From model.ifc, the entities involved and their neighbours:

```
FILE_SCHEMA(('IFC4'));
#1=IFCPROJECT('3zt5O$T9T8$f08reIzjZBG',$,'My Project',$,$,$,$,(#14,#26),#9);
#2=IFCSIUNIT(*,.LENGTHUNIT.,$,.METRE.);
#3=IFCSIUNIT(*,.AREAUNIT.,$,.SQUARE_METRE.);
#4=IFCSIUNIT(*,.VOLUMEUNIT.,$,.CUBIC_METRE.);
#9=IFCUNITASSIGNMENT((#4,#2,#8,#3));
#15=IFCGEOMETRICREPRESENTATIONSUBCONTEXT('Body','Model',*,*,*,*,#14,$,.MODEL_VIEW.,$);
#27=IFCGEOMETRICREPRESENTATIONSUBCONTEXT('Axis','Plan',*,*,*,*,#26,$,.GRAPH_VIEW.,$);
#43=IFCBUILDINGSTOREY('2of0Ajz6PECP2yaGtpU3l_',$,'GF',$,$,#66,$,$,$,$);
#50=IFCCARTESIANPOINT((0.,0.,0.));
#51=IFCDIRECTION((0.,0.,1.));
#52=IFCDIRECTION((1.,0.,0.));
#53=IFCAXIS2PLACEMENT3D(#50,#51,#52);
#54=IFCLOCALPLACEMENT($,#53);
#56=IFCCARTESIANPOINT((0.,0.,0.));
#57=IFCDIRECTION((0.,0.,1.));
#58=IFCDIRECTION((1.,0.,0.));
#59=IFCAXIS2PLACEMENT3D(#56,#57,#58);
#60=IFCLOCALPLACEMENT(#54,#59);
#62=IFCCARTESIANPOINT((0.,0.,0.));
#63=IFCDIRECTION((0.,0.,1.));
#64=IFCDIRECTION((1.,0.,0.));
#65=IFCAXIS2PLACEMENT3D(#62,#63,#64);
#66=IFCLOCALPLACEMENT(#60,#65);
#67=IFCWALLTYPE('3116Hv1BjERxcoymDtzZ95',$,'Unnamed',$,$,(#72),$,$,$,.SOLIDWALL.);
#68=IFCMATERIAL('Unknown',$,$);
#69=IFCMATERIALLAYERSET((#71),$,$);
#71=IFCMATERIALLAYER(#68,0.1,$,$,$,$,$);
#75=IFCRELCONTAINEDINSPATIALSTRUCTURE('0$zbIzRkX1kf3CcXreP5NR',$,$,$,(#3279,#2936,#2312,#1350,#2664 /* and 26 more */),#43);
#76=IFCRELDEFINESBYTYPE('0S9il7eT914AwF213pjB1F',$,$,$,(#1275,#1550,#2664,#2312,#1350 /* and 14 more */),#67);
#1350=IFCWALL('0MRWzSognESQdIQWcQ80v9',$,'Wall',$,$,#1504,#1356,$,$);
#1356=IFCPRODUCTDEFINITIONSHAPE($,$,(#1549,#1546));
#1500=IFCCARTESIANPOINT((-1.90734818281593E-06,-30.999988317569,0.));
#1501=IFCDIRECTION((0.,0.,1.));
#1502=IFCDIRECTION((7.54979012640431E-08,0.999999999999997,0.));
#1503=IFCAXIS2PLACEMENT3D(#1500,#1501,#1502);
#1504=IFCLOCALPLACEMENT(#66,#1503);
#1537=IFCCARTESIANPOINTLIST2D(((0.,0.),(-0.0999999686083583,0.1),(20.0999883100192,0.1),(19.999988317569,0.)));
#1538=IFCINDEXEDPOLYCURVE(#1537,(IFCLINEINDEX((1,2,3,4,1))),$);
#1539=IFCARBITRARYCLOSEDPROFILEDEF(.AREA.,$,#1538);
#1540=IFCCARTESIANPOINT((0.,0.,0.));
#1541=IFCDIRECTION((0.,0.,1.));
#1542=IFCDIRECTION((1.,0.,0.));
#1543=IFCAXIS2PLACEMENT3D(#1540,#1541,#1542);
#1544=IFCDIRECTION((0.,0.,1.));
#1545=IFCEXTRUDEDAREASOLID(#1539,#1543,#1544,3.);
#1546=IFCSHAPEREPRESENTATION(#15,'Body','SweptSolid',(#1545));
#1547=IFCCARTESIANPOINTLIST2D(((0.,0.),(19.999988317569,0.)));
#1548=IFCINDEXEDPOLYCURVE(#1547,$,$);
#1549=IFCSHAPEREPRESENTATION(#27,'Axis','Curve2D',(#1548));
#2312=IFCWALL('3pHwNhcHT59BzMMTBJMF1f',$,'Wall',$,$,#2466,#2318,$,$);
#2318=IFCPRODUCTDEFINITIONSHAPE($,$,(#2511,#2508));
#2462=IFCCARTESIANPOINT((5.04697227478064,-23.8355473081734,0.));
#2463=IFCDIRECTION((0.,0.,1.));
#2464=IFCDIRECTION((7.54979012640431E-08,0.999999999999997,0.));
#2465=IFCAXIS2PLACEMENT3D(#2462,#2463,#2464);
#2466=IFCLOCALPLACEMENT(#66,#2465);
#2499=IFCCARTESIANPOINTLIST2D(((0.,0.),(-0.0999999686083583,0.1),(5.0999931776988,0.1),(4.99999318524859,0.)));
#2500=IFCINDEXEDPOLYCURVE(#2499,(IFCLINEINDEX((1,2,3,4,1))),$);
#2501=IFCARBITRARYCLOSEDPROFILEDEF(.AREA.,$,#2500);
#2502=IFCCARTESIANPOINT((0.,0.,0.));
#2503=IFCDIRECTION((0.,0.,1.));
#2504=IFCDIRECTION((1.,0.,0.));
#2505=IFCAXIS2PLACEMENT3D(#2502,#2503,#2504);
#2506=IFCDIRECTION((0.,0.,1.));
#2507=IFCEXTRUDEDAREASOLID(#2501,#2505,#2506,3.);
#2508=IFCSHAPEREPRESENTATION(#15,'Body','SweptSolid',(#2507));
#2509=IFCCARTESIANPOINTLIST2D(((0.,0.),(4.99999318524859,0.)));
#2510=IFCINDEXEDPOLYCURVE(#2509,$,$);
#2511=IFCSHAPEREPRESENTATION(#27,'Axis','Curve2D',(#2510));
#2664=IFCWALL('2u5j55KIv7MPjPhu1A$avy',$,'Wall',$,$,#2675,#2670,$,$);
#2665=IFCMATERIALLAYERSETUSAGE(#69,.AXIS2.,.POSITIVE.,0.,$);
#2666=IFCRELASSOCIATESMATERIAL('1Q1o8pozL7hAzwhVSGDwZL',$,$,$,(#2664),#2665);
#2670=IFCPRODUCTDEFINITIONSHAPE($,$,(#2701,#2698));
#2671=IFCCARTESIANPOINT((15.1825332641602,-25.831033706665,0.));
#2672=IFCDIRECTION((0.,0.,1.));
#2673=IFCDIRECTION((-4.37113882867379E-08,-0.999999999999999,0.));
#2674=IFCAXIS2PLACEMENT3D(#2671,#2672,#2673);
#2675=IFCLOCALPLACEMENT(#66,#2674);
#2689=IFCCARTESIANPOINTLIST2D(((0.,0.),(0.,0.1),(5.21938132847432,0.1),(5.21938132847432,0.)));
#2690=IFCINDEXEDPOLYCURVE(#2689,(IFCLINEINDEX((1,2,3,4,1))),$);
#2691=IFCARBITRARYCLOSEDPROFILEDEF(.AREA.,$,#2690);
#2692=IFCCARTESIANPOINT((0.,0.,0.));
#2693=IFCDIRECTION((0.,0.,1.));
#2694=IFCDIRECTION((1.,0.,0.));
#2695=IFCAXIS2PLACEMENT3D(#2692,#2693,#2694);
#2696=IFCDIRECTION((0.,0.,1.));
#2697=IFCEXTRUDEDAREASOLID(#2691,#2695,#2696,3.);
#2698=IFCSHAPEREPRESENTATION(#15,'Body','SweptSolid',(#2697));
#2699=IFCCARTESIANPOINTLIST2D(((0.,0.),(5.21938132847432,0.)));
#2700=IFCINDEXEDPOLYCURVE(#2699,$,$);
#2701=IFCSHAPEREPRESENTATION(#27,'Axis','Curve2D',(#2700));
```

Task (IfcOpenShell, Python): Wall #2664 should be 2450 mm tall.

```python
import ifcopenshell
import ifcopenshell.geom
import ifcopenshell.util.representation
import ifcopenshell.util.shape
import ifcopenshell.util.unit

model = ifcopenshell.open("model.ifc")
unit_scale = ifcopenshell.util.unit.calculate_unit_scale(model)
settings = ifcopenshell.geom.settings()


def volume(element):
    """Net volume in cubic metres, openings subtracted."""
    shape = ifcopenshell.geom.create_shape(settings, element)
    return ifcopenshell.util.shape.get_volume(shape.geometry)


wall = model.by_guid("2u5j55KIv7MPjPhu1A$avy")
before = volume(wall)

body = ifcopenshell.util.representation.get_representation(wall, "Model", "Body")
solid = body.Items[0]
old_height = solid.Depth
solid.Depth = 2.45 / unit_scale
after = volume(wall)

print(f"height {old_height:g} -> {solid.Depth:g}, volume {before:.3f} -> {after:.3f} m3")

model.write("model_v2.ifc")
```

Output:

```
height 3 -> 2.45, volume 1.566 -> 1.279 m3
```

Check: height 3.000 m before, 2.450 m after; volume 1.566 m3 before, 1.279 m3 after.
